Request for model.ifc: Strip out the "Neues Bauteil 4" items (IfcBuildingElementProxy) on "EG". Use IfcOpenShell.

First a look at what the model holds.

```python
import ifcopenshell
import ifcopenshell.util.element

model = ifcopenshell.open("model.ifc")
print(model.schema)
storey = next(s for s in model.by_type("IfcBuildingStorey") if s.Name == "EG")
proxies = [e for e in ifcopenshell.util.element.get_decomposition(storey) if e.is_a("IfcBuildingElementProxy")]
seen = {}
for e in proxies:
    element_type = ifcopenshell.util.element.get_type(e)
    name = element_type.Name if element_type not in (None, e) else None
    seen[name] = seen.get(name, 0) + 1
for name, count in sorted(seen.items(), key=str):
    print(count, "x", name)
```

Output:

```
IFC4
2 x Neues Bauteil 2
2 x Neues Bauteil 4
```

```python
import ifcopenshell
import ifcopenshell.api.root
import ifcopenshell.util.element

model = ifcopenshell.open("model.ifc")

storey = next(s for s in model.by_type("IfcBuildingStorey") if s.Name == "EG")
proxies = [e for e in ifcopenshell.util.element.get_decomposition(storey) if e.is_a("IfcBuildingElementProxy")]
targets = [e for e in proxies if (t := ifcopenshell.util.element.get_type(e)) not in (None, e) and t.Name == "Neues Bauteil 4"]

for e in targets:
    ifcopenshell.api.root.remove_product(model, product=e)
print(len(targets), "removed")

model.write("model_v2.ifc")
```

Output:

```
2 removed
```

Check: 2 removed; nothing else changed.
